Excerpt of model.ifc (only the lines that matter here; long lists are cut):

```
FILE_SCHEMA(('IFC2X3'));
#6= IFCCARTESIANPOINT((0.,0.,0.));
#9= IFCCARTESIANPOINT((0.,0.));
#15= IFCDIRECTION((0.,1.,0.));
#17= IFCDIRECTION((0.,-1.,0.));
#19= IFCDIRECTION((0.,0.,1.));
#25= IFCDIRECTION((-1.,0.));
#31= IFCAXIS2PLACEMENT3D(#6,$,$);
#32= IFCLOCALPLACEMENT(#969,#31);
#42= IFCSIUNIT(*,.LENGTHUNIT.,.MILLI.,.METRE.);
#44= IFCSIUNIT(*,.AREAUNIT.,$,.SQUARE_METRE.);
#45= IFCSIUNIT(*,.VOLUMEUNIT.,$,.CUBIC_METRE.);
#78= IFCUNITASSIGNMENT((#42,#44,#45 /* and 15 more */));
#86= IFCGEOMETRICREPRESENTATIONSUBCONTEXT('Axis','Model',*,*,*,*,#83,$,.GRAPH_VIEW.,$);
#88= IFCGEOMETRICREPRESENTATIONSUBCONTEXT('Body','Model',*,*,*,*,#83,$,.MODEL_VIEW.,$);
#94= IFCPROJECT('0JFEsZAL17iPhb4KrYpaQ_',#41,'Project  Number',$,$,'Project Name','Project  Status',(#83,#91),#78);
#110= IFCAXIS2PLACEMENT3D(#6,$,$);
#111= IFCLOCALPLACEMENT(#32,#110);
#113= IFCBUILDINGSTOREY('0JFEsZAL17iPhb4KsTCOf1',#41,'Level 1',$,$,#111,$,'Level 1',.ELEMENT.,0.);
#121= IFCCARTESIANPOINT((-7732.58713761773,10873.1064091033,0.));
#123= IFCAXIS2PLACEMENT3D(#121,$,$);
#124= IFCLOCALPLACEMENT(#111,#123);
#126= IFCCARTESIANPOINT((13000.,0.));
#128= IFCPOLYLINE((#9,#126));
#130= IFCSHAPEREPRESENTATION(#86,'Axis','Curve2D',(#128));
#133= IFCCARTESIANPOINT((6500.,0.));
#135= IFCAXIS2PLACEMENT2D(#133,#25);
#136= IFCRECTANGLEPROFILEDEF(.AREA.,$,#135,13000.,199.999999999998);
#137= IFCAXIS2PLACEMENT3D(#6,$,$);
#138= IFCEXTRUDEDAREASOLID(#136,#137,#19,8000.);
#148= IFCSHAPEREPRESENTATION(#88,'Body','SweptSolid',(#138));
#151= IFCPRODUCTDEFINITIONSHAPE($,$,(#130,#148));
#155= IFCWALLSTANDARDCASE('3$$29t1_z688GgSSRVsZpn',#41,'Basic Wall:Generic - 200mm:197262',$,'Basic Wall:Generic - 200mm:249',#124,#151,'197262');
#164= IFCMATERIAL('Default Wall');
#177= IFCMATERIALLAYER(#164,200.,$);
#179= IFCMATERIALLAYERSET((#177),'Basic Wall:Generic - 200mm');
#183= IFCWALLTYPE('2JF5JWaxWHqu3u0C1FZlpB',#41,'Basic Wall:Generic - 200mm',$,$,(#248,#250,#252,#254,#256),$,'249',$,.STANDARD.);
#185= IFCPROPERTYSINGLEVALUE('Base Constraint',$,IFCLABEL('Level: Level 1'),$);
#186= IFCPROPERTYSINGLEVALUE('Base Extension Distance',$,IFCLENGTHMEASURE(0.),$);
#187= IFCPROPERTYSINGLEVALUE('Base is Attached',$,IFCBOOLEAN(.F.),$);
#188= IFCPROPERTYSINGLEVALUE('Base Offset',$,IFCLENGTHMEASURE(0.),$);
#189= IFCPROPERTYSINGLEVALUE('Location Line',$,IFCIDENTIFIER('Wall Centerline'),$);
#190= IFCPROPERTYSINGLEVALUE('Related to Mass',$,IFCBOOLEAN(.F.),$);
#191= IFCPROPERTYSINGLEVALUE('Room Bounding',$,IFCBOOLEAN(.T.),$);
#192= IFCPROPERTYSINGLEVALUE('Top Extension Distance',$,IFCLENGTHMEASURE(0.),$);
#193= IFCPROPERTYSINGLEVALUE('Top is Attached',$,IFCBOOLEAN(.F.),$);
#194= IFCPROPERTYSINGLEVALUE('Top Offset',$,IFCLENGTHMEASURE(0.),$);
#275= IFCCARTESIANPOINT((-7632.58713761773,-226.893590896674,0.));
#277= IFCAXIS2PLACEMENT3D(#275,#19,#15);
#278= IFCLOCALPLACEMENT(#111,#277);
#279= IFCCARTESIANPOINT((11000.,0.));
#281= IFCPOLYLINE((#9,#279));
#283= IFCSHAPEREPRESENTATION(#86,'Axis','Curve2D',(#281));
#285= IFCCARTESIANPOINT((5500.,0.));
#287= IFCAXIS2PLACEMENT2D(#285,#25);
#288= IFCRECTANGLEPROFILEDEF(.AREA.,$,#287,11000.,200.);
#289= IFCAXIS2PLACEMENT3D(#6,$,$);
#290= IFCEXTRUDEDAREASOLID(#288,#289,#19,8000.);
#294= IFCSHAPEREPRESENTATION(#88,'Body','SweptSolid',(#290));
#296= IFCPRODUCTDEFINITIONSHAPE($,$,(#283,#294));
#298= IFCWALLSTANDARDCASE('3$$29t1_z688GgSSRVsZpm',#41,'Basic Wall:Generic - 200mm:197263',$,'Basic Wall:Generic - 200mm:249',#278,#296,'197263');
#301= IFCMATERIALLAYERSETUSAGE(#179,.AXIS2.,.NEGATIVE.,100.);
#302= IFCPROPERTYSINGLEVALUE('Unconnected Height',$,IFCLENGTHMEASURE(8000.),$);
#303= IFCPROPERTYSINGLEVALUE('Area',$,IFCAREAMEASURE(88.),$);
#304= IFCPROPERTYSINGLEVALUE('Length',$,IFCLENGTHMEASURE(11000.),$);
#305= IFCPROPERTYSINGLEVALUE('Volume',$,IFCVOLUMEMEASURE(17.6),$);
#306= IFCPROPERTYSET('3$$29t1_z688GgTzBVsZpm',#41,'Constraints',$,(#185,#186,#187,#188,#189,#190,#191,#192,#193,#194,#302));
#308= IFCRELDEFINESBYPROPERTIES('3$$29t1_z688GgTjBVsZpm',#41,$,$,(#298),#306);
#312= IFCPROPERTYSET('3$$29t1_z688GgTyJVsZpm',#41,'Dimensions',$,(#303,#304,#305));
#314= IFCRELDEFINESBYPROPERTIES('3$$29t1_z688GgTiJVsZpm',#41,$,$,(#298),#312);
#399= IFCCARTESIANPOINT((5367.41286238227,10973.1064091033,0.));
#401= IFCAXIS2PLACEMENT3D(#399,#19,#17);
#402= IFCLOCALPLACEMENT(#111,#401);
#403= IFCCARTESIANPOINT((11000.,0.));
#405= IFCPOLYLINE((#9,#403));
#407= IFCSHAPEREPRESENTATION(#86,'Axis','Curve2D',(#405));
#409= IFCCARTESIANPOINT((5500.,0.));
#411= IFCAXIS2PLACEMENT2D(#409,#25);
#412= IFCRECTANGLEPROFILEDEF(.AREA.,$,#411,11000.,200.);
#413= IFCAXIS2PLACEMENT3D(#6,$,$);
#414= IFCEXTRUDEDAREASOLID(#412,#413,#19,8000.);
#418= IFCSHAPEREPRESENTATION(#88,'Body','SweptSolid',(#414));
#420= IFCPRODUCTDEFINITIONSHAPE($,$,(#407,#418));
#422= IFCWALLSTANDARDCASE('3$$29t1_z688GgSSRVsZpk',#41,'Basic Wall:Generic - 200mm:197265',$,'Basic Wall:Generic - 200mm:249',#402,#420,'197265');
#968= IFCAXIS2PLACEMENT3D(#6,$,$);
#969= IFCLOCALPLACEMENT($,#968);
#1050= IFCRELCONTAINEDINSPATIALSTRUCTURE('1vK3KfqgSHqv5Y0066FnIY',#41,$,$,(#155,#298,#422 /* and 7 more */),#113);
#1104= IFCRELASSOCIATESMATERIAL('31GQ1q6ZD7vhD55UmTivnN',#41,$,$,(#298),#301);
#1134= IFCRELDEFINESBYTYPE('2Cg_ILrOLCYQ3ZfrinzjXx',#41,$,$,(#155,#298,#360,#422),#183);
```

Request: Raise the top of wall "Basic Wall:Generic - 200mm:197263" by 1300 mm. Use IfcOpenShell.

```python
import ifcopenshell
import ifcopenshell.api.pset
import ifcopenshell.geom
import ifcopenshell.util.element
import ifcopenshell.util.representation
import ifcopenshell.util.shape
import ifcopenshell.util.unit

model = ifcopenshell.open("model.ifc")
unit_scale = ifcopenshell.util.unit.calculate_unit_scale(model)
area_scale = ifcopenshell.util.unit.calculate_unit_scale(model, "AREAUNIT")
volume_scale = ifcopenshell.util.unit.calculate_unit_scale(model, "VOLUMEUNIT")
settings = ifcopenshell.geom.settings()


def volume(element):
    """Net volume in cubic metres, openings subtracted."""
    shape = ifcopenshell.geom.create_shape(settings, element)
    return ifcopenshell.util.shape.get_volume(shape.geometry)


wall = model.by_guid("3$$29t1_z688GgSSRVsZpm")
before = volume(wall)

body = ifcopenshell.util.representation.get_representation(wall, "Model", "Body")
solid = body.Items[0]
old_height = solid.Depth
solid.Depth += 1.3 / unit_scale
after = volume(wall)
thickness = 0.2  # wall thickness in metres

# Update the stored height, areas and volumes.
pset = model.by_id(ifcopenshell.util.element.get_pset(wall, "Constraints", should_inherit=False)["id"])
ifcopenshell.api.pset.edit_pset(model, pset=pset, properties={
    "Unconnected Height": model.create_entity("IfcLengthMeasure", solid.Depth),
})
pset = model.by_id(ifcopenshell.util.element.get_pset(wall, "Dimensions", should_inherit=False)["id"])
ifcopenshell.api.pset.edit_pset(model, pset=pset, properties={
    "Area": model.create_entity("IfcAreaMeasure", after / thickness / area_scale),
    "Volume": model.create_entity("IfcVolumeMeasure", after / volume_scale),
})

print(f"height {old_height:g} -> {solid.Depth:g}, volume {before:.3f} -> {after:.3f} m3")

model.write("model_updated.ifc")
```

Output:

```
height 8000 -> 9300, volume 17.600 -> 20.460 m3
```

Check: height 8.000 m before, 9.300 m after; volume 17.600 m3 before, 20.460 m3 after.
